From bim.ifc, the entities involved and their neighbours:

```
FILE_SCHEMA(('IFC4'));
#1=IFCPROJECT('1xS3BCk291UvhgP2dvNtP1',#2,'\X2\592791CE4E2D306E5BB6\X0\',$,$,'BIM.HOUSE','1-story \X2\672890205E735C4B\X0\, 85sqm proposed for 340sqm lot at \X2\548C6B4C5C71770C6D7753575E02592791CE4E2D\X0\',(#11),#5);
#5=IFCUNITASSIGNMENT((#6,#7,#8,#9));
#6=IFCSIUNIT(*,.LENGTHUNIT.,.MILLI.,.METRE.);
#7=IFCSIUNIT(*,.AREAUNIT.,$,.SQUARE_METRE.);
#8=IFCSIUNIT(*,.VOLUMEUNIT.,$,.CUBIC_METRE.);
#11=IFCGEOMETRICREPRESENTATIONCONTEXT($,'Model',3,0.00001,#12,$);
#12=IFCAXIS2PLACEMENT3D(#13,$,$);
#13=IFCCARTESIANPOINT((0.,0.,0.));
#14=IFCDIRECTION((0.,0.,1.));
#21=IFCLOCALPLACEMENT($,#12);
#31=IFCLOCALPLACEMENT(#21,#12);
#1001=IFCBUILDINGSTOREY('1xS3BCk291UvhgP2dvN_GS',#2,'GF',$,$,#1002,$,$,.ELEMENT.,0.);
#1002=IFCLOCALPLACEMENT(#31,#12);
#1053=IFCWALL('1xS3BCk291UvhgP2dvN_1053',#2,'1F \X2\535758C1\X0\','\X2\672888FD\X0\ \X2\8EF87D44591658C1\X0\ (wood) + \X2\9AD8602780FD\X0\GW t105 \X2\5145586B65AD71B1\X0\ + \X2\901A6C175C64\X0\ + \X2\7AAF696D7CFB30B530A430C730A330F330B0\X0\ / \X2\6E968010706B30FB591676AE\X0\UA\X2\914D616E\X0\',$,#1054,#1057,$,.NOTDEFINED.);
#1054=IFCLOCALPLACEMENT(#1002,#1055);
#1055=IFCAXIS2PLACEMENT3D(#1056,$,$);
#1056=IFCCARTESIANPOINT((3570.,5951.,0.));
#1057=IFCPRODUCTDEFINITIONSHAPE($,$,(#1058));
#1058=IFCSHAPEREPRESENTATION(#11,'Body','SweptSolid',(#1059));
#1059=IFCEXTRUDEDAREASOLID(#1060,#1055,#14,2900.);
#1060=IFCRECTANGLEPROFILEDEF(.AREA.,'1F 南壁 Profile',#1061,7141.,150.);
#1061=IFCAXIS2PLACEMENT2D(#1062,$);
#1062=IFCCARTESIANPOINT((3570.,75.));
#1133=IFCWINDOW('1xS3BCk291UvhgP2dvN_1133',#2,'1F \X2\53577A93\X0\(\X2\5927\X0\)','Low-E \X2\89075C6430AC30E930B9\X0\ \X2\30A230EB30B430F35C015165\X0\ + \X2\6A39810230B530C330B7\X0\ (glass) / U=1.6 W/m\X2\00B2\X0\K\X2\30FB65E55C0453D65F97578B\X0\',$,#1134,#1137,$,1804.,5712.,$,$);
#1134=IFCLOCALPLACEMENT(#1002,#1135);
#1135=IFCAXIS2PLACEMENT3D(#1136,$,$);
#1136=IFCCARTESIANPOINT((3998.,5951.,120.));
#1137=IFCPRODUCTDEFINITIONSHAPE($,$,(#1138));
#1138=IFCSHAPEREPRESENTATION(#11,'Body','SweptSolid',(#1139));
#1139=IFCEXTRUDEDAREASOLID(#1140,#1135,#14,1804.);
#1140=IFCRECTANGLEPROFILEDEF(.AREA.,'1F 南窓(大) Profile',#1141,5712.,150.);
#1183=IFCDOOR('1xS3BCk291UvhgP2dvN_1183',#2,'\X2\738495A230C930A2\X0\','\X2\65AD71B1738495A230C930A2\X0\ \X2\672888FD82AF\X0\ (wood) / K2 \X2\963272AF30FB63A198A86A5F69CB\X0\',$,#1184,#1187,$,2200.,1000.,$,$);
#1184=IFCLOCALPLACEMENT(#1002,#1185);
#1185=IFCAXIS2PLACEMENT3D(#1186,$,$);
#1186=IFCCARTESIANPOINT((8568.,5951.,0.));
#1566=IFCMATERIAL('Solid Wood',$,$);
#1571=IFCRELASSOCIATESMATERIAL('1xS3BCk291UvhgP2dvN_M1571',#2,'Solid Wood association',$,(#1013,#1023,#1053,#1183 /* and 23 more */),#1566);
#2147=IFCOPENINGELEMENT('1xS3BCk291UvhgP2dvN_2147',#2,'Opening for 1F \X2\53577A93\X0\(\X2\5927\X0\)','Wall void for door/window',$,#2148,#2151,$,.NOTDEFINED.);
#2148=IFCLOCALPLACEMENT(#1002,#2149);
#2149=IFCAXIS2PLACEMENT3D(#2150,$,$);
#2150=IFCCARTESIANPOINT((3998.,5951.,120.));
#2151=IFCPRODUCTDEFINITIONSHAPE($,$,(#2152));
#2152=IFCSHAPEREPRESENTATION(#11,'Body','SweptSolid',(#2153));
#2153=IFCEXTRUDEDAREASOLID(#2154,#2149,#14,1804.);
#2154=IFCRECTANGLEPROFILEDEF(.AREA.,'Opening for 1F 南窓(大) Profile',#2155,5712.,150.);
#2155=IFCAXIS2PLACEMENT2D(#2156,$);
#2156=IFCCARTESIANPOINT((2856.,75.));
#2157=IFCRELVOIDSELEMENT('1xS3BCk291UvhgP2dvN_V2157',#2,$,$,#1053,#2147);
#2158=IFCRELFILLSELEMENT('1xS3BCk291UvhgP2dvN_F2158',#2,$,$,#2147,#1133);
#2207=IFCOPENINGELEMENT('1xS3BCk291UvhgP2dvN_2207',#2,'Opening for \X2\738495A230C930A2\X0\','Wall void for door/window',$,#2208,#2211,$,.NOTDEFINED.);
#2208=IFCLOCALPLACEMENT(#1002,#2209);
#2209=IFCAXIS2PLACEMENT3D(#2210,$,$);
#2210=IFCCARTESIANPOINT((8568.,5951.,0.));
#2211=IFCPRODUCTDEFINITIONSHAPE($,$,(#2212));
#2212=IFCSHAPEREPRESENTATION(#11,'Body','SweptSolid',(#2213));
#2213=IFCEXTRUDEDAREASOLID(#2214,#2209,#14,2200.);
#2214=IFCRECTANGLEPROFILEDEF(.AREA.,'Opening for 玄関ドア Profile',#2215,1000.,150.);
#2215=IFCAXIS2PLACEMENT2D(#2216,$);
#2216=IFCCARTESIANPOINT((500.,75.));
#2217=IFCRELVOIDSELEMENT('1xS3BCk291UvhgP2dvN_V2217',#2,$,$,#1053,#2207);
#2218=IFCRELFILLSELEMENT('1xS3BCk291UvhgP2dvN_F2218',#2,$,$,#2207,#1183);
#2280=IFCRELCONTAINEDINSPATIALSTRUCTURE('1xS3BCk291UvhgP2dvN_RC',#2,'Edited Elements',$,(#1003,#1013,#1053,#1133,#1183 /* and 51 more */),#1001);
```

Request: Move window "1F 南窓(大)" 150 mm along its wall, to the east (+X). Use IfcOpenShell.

```python
import ifcopenshell
import ifcopenshell.api.geometry
import ifcopenshell.util.placement
import ifcopenshell.util.unit

model = ifcopenshell.open("bim.ifc")
unit_scale = ifcopenshell.util.unit.calculate_unit_scale(model)

window = model.by_guid("1xS3BCk291UvhgP2dvN_1133")
opening = window.FillsVoids[0].RelatingOpeningElement
wall = opening.VoidsElements[0].RelatingBuildingElement

wall_matrix = ifcopenshell.util.placement.get_local_placement(wall.ObjectPlacement)
shift = wall_matrix[:3, 0] * 0.15 / unit_scale
before = ifcopenshell.util.placement.get_local_placement(window.ObjectPlacement)[:3, 3].copy()

# The window is not placed relative to its opening, so move both.
for product in (opening, window):
    matrix = ifcopenshell.util.placement.get_local_placement(product.ObjectPlacement)
    matrix[:3, 3] += shift
    ifcopenshell.api.geometry.edit_object_placement(model, product=product, matrix=matrix, is_si=False)

after = ifcopenshell.util.placement.get_local_placement(window.ObjectPlacement)[:3, 3]
print("window moved by", (after - before).round(3) + 0.0)

model.write("bim-out.ifc")
```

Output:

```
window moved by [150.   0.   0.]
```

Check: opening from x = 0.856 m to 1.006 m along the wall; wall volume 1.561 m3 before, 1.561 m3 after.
